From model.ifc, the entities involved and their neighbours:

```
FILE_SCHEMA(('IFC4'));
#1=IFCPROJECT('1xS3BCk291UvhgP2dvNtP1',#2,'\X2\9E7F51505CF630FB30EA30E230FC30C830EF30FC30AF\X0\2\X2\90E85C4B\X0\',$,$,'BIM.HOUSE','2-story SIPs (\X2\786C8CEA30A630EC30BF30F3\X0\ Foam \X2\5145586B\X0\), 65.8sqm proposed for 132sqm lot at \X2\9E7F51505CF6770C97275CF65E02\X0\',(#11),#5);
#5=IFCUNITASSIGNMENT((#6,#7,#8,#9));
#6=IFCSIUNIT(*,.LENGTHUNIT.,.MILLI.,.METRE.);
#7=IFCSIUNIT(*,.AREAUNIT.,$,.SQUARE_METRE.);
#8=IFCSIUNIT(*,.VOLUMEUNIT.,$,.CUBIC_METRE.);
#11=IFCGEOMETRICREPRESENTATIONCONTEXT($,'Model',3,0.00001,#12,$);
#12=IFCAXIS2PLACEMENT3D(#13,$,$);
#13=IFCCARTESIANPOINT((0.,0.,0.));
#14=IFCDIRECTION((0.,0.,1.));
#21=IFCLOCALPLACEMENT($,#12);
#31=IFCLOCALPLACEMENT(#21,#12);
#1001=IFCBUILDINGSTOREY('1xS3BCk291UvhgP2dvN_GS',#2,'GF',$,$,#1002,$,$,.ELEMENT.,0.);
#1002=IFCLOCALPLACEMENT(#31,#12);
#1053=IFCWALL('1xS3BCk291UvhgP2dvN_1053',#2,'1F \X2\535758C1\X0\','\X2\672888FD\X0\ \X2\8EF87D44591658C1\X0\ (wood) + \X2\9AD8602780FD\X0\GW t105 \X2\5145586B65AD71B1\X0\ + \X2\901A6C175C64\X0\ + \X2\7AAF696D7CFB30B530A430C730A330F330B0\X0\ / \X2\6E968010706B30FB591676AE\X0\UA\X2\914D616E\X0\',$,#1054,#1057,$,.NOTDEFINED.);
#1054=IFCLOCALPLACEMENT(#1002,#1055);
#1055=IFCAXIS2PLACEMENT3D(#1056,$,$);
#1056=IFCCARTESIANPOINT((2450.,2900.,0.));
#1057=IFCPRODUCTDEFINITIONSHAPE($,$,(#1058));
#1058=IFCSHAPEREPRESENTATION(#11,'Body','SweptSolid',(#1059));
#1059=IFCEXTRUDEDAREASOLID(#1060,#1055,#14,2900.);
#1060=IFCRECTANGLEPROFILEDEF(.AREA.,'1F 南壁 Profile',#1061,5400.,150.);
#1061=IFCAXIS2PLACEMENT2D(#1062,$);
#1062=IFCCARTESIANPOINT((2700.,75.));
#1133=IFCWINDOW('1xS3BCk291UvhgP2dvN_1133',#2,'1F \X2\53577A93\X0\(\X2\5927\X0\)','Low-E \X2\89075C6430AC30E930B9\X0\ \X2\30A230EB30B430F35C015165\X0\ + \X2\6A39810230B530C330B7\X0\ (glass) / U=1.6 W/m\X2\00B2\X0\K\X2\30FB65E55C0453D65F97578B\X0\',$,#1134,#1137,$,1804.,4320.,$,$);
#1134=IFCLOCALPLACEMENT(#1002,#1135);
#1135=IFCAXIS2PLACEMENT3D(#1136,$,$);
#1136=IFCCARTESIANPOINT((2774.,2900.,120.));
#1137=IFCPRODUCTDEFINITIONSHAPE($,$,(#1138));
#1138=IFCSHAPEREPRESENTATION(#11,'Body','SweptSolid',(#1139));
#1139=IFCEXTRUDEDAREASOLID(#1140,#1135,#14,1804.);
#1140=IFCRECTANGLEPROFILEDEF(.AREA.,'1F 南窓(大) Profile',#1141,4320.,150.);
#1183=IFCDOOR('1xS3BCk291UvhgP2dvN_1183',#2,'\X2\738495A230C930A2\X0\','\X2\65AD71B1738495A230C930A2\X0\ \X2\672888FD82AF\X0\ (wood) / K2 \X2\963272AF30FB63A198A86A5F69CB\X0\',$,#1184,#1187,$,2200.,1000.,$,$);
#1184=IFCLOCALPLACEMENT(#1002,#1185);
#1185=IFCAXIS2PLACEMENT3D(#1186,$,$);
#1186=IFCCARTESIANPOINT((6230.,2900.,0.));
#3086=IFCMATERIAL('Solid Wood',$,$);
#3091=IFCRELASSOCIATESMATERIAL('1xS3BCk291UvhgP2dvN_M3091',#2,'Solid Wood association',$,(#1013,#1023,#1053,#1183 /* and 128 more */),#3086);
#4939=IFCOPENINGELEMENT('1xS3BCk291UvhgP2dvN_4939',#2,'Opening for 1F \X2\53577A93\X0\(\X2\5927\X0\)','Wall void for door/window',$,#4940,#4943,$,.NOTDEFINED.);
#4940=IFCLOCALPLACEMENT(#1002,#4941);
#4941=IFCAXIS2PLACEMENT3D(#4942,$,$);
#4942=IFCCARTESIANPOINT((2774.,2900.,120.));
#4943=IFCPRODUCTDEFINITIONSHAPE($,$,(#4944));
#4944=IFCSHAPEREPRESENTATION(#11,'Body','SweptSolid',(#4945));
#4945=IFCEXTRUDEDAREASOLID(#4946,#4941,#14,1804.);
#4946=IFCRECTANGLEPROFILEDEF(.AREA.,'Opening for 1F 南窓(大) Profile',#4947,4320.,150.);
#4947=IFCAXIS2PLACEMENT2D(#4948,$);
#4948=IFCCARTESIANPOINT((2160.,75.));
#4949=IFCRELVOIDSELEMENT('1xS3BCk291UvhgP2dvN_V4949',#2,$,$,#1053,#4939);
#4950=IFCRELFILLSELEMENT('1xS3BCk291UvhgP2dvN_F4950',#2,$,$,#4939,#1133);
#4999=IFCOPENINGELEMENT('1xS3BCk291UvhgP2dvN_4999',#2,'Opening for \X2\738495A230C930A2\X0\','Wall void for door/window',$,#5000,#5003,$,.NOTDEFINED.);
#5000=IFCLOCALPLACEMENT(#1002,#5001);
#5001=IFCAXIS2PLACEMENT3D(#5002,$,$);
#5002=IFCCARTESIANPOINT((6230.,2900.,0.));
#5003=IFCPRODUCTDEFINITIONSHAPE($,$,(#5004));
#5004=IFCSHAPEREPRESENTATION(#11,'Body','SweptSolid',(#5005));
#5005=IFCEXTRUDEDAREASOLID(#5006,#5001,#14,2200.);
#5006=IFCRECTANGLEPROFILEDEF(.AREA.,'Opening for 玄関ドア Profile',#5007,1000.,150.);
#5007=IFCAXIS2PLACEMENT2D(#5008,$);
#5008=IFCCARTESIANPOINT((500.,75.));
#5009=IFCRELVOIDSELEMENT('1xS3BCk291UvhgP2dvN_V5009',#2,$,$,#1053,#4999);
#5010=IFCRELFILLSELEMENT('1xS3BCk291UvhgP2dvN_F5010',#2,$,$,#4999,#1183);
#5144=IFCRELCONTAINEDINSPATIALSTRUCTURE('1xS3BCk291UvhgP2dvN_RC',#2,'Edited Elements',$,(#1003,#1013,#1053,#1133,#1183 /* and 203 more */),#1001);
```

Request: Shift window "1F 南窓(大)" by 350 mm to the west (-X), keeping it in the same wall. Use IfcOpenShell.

```python
import ifcopenshell
import ifcopenshell.api.geometry
import ifcopenshell.util.placement
import ifcopenshell.util.unit

model = ifcopenshell.open("model.ifc")
unit_scale = ifcopenshell.util.unit.calculate_unit_scale(model)

window = model.by_guid("1xS3BCk291UvhgP2dvN_1133")
opening = window.FillsVoids[0].RelatingOpeningElement
wall = opening.VoidsElements[0].RelatingBuildingElement

wall_matrix = ifcopenshell.util.placement.get_local_placement(wall.ObjectPlacement)
shift = wall_matrix[:3, 0] * -0.35 / unit_scale
before = ifcopenshell.util.placement.get_local_placement(window.ObjectPlacement)[:3, 3].copy()

# The window is not placed relative to its opening, so move both.
for product in (opening, window):
    matrix = ifcopenshell.util.placement.get_local_placement(product.ObjectPlacement)
    matrix[:3, 3] += shift
    ifcopenshell.api.geometry.edit_object_placement(model, product=product, matrix=matrix, is_si=False)

after = ifcopenshell.util.placement.get_local_placement(window.ObjectPlacement)[:3, 3]
print("window moved by", (after - before).round(3) + 0.0)

model.write("model_v2.ifc")
```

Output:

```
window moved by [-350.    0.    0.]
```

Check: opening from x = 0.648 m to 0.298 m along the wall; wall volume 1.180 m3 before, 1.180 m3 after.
